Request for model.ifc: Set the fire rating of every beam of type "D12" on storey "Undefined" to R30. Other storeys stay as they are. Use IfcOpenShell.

First a look at what the model holds.

```python
import ifcopenshell
import ifcopenshell.util.element

model = ifcopenshell.open("model.ifc")
print(model.schema)
storey = next(s for s in model.by_type("IfcBuildingStorey") if s.Name == "Undefined")
beams = [e for e in ifcopenshell.util.element.get_decomposition(storey) if e.is_a("IfcBeam")]
seen = {}
for e in beams:
    element_type = ifcopenshell.util.element.get_type(e)
    key = (element_type.Name if element_type != e and element_type else None, ifcopenshell.util.element.get_pset(e, "Pset_BeamCommon", "FireRating"))
    seen[key] = seen.get(key, 0) + 1
for (name, value), count in sorted(seen.items(), key=str):
    print(count, "x", name, "|", value)
```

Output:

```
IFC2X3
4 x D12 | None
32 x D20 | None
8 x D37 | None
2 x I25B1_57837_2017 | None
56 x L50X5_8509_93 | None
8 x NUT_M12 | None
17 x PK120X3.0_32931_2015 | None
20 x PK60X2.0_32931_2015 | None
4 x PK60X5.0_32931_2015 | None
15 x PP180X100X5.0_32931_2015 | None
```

```python
import ifcopenshell
import ifcopenshell.api.pset
import ifcopenshell.util.element

model = ifcopenshell.open("model.ifc")

storey = next(s for s in model.by_type("IfcBuildingStorey") if s.Name == "Undefined")
beams = [e for e in ifcopenshell.util.element.get_decomposition(storey) if e.is_a("IfcBeam")]

count = 0
for e in beams:
    element_type = ifcopenshell.util.element.get_type(e)
    if element_type in (None, e) or element_type.Name != "D12":
        continue
    found = ifcopenshell.util.element.get_pset(e, "Pset_BeamCommon", should_inherit=False)
    if found:
        pset = model.by_id(found["id"])
        if len(ifcopenshell.util.element.get_elements_by_pset(pset)) > 1:
            pset = ifcopenshell.api.pset.unshare_pset(model, products=[e], pset=pset)[0]
    else:
        pset = ifcopenshell.api.pset.add_pset(model, product=e, name="Pset_BeamCommon")
    ifcopenshell.api.pset.edit_pset(model, pset=pset, properties={"FireRating": "R30"})
    count += 1

print(count, "beams updated")

model.write("model_rev.ifc")
```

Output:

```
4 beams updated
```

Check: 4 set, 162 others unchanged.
